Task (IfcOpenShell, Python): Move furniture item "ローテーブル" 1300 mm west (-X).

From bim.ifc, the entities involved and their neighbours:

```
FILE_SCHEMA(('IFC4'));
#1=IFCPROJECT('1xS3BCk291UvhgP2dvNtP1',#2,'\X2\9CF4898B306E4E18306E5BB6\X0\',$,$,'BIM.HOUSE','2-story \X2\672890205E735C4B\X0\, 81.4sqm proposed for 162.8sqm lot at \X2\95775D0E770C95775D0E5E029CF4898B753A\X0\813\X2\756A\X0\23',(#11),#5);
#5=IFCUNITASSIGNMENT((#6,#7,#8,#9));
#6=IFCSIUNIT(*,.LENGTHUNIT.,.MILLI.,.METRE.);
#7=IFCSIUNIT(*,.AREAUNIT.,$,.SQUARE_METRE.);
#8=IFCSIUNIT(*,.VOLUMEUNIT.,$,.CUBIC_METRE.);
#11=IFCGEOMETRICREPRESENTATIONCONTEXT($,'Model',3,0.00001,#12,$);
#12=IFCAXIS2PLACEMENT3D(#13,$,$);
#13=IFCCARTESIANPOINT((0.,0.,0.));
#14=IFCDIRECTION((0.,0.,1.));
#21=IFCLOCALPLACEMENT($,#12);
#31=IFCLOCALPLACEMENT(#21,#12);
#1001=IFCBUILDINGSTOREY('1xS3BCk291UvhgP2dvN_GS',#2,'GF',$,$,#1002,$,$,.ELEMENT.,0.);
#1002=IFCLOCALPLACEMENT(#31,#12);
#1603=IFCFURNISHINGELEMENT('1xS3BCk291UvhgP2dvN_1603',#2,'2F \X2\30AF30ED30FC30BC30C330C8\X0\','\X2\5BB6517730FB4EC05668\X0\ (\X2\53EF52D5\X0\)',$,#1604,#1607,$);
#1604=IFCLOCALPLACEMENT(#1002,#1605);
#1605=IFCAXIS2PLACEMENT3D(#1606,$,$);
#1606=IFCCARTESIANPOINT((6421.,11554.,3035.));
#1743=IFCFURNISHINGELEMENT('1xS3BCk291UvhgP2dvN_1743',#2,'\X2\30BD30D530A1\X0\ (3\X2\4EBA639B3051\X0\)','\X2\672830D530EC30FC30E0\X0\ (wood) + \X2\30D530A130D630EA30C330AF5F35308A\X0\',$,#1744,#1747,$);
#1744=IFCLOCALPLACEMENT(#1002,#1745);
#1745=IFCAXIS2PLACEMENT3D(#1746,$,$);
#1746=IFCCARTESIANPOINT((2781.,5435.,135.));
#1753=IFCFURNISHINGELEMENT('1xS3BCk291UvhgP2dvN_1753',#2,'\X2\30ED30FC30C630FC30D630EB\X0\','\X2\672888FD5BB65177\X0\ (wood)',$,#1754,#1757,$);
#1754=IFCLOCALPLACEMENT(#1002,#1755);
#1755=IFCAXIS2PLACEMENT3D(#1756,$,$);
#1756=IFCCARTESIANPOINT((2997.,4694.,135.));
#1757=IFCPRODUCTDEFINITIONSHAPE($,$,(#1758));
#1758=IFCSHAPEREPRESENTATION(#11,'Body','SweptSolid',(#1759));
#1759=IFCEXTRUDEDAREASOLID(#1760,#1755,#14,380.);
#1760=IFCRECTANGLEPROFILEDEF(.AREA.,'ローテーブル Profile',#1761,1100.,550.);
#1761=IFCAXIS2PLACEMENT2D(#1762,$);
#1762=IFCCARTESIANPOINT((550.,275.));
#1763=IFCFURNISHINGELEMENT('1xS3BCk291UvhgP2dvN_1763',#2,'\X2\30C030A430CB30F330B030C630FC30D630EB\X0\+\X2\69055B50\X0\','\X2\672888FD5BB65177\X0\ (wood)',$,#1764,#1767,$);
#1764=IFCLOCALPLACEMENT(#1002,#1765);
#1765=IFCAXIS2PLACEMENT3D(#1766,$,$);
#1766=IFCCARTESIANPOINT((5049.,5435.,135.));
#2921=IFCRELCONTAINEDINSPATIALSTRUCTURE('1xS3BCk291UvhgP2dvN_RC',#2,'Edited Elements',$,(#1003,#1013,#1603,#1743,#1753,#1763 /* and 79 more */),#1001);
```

```python
import ifcopenshell
import ifcopenshell.api.geometry
import ifcopenshell.util.placement
import ifcopenshell.util.unit

model = ifcopenshell.open("bim.ifc")
unit_scale = ifcopenshell.util.unit.calculate_unit_scale(model)

item = model.by_guid("1xS3BCk291UvhgP2dvN_1753")
matrix = ifcopenshell.util.placement.get_local_placement(item.ObjectPlacement)
matrix[0, 3] -= 1.3 / unit_scale
ifcopenshell.api.geometry.edit_object_placement(model, product=item, matrix=matrix, is_si=False)

print(ifcopenshell.util.placement.get_local_placement(item.ObjectPlacement).round(3) + 0.0)

model.write("bim_edited.ifc")
```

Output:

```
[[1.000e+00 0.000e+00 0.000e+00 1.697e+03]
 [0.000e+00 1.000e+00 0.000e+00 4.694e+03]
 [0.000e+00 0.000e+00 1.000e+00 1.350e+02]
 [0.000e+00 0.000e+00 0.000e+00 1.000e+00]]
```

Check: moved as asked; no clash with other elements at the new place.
